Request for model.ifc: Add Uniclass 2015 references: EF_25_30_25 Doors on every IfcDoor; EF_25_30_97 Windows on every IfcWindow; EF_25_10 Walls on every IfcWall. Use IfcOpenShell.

First a look at what the model holds.

```python
import ifcopenshell

model = ifcopenshell.open("model.ifc")
print(model.schema)
print("classifications:", [c.Name for c in model.by_type("IfcClassification")])
for ifc_class in ("IfcDoor", "IfcRoof", "IfcStair", "IfcWall", "IfcWindow"):
    print(ifc_class, len(model.by_type(ifc_class)))
```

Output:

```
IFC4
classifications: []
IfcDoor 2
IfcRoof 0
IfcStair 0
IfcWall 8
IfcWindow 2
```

```python
import ifcopenshell
import ifcopenshell.api.classification

model = ifcopenshell.open("model.ifc")

system = ifcopenshell.api.classification.add_classification(model, classification="Uniclass 2015")

codes = {
    "IfcDoor": ("EF_25_30_25", "Doors"),
    "IfcWindow": ("EF_25_30_97", "Windows"),
    "IfcWall": ("EF_25_10", "Walls"),
}
for ifc_class, (code, name) in codes.items():
    products = model.by_type(ifc_class)
    ifcopenshell.api.classification.add_reference(
        model, products=products, classification=system, identification=code, name=name
    )
    print(code, len(products))

model.write("model-out.ifc")
```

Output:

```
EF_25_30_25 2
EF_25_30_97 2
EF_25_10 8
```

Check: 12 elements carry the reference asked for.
